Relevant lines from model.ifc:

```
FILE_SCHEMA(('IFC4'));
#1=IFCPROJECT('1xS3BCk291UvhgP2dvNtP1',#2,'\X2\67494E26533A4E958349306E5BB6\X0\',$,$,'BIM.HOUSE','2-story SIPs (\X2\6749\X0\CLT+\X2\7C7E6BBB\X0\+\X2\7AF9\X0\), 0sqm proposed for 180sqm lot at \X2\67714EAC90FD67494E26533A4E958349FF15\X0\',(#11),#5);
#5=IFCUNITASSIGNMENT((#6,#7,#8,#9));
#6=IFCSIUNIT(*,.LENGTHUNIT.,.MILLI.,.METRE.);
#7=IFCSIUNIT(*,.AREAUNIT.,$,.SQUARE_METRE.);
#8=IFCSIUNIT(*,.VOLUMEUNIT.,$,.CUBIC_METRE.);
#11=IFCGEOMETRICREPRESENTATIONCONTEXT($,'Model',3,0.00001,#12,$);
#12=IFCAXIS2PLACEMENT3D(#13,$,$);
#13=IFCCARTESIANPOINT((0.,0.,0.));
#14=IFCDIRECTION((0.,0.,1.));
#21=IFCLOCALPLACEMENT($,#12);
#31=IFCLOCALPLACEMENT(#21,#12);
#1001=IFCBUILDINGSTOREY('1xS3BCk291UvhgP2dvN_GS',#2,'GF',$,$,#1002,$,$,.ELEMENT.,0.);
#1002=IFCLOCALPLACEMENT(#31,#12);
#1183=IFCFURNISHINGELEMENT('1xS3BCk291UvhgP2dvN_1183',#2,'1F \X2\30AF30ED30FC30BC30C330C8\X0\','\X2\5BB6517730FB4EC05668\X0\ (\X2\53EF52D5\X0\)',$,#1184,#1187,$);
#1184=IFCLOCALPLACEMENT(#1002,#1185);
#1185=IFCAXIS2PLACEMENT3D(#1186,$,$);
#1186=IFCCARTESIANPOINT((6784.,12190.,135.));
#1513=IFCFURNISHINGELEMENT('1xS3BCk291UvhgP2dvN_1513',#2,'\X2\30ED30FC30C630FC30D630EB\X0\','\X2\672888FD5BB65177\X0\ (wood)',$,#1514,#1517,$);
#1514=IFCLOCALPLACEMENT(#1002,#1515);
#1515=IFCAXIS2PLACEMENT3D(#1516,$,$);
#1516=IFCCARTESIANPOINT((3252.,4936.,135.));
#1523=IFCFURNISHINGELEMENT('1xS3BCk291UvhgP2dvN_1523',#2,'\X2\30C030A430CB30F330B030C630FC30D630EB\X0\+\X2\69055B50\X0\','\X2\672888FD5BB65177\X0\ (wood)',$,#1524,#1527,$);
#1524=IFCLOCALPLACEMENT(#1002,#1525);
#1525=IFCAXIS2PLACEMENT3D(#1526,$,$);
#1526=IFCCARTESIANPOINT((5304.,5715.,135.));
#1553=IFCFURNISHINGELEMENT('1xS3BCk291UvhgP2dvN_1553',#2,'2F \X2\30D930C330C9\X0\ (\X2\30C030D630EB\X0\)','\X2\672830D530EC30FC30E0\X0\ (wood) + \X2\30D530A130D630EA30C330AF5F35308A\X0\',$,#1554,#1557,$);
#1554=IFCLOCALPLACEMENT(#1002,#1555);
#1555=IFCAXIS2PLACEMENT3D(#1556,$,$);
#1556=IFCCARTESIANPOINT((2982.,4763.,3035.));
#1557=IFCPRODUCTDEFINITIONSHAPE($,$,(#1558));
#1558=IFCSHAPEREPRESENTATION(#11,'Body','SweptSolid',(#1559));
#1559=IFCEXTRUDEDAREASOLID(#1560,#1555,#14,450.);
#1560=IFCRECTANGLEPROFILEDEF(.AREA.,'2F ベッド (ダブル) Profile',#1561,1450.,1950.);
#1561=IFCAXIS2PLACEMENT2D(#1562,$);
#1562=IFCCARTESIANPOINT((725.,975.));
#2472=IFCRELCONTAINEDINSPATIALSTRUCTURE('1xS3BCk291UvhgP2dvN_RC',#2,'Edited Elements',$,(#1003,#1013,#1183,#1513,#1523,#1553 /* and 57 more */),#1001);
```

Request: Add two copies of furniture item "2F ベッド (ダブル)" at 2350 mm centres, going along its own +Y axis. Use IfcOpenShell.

```python
import ifcopenshell
import ifcopenshell.api.geometry
import ifcopenshell.api.root
import ifcopenshell.util.element
import ifcopenshell.util.placement
import ifcopenshell.util.unit

model = ifcopenshell.open("model.ifc")
unit_scale = ifcopenshell.util.unit.calculate_unit_scale(model)


def reuse_history(source, copy):
    """copy_class also copies each property set's owner history, people and application; keep the originals."""
    for rel in copy.IsDefinedBy:
        if rel.is_a("IfcRelDefinesByProperties") and (history := rel.RelatingPropertyDefinition.OwnerHistory):
            rel.RelatingPropertyDefinition.OwnerHistory = source.OwnerHistory
            ifcopenshell.util.element.remove_deep2(model, history)


source = model.by_id(1553)
base = ifcopenshell.util.placement.get_local_placement(source.ObjectPlacement)
step = base[:3, 1] * 2.35 / unit_scale

for i in range(1, 3):
    copy = ifcopenshell.api.root.copy_class(model, product=source)
    copy.Representation = ifcopenshell.util.element.copy_deep(
        model, source.Representation, exclude=["IfcGeometricRepresentationContext", "IfcRepresentationMap"]
    )
    reuse_history(source, copy)
    matrix = base.copy()
    matrix[:3, 3] += i * step
    print("added at", matrix[:3, 3].round(3) + 0.0)
    ifcopenshell.api.geometry.edit_object_placement(model, product=copy, matrix=matrix, is_si=False)

model.write("model_edited.ifc")
```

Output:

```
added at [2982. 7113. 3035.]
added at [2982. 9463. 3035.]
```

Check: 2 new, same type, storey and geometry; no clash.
